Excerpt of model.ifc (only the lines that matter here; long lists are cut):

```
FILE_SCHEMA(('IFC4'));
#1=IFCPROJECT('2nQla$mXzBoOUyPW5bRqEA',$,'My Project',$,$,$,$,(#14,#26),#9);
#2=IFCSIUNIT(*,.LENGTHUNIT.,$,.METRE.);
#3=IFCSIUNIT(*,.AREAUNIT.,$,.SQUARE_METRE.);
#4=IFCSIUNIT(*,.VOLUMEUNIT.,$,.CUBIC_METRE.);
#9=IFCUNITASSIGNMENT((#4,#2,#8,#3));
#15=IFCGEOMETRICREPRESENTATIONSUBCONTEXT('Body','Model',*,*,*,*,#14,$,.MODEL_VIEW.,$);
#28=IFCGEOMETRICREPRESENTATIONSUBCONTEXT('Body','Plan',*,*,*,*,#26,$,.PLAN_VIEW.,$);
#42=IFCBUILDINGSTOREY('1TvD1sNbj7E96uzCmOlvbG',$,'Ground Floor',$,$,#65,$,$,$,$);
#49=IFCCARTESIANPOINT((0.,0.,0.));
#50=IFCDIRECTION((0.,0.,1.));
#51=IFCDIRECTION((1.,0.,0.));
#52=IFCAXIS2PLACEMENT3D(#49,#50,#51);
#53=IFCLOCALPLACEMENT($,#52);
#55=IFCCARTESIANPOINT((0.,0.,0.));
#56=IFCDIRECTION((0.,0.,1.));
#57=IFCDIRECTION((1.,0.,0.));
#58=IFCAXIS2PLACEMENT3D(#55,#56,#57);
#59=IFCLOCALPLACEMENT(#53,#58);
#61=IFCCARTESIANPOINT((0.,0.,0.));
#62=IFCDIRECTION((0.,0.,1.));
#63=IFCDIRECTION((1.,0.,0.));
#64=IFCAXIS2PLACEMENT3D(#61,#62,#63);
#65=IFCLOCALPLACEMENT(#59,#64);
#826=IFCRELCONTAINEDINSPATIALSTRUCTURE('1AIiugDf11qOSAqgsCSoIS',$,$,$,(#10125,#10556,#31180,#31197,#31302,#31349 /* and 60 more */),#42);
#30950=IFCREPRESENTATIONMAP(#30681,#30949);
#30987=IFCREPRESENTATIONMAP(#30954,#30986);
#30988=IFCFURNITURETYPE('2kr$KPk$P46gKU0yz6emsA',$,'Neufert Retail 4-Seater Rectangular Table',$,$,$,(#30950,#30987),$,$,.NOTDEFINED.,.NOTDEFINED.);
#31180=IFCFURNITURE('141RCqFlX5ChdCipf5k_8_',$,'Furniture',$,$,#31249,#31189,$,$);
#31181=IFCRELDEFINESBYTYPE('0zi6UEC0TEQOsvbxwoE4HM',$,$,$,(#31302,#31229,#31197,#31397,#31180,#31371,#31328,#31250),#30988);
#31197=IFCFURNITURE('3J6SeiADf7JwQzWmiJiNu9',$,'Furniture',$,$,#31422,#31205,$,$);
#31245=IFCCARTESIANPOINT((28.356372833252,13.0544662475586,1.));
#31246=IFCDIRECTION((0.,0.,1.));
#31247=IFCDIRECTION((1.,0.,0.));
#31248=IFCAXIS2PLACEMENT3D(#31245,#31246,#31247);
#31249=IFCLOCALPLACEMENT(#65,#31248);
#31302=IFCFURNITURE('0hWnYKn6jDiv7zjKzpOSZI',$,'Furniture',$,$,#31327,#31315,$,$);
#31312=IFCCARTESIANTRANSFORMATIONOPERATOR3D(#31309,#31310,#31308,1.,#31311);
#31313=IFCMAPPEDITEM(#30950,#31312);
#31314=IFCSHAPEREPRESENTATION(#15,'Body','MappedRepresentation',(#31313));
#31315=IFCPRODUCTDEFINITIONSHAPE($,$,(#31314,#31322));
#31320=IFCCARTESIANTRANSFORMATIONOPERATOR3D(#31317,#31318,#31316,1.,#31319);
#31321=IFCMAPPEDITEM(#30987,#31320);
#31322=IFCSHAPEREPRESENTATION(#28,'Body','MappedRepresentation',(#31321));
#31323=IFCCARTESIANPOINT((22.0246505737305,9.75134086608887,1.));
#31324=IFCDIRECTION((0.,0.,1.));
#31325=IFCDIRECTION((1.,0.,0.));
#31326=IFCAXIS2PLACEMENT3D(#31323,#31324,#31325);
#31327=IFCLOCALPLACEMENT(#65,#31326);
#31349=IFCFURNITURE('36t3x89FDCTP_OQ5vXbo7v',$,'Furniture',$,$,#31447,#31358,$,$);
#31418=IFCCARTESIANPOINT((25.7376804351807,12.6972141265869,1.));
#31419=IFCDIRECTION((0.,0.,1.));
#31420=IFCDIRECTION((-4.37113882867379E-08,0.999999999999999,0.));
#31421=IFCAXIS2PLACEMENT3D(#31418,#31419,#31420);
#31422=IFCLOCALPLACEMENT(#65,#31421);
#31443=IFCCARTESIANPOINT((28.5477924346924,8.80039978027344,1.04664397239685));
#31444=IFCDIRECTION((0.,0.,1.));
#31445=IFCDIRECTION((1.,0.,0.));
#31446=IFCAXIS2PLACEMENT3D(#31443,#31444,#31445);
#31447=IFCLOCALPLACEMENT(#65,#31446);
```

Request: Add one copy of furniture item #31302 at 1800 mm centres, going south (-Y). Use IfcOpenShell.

```python
import numpy as np
import ifcopenshell
import ifcopenshell.api.geometry
import ifcopenshell.api.root
import ifcopenshell.util.element
import ifcopenshell.util.placement
import ifcopenshell.util.unit

model = ifcopenshell.open("model.ifc")
unit_scale = ifcopenshell.util.unit.calculate_unit_scale(model)

source = model.by_guid("0hWnYKn6jDiv7zjKzpOSZI")
base = ifcopenshell.util.placement.get_local_placement(source.ObjectPlacement)
step = np.array([0.0, -1.0, 0.0]) * 1.8 / unit_scale

for i in range(1, 2):
    copy = ifcopenshell.api.root.copy_class(model, product=source)
    copy.Representation = ifcopenshell.util.element.copy_deep(
        model, source.Representation, exclude=["IfcGeometricRepresentationContext", "IfcRepresentationMap"]
    )
    matrix = base.copy()
    matrix[:3, 3] += i * step
    print("added at", matrix[:3, 3].round(3) + 0.0)
    ifcopenshell.api.geometry.edit_object_placement(model, product=copy, matrix=matrix, is_si=False)

model.write("model-out.ifc")
```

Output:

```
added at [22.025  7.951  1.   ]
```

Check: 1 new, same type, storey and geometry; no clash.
